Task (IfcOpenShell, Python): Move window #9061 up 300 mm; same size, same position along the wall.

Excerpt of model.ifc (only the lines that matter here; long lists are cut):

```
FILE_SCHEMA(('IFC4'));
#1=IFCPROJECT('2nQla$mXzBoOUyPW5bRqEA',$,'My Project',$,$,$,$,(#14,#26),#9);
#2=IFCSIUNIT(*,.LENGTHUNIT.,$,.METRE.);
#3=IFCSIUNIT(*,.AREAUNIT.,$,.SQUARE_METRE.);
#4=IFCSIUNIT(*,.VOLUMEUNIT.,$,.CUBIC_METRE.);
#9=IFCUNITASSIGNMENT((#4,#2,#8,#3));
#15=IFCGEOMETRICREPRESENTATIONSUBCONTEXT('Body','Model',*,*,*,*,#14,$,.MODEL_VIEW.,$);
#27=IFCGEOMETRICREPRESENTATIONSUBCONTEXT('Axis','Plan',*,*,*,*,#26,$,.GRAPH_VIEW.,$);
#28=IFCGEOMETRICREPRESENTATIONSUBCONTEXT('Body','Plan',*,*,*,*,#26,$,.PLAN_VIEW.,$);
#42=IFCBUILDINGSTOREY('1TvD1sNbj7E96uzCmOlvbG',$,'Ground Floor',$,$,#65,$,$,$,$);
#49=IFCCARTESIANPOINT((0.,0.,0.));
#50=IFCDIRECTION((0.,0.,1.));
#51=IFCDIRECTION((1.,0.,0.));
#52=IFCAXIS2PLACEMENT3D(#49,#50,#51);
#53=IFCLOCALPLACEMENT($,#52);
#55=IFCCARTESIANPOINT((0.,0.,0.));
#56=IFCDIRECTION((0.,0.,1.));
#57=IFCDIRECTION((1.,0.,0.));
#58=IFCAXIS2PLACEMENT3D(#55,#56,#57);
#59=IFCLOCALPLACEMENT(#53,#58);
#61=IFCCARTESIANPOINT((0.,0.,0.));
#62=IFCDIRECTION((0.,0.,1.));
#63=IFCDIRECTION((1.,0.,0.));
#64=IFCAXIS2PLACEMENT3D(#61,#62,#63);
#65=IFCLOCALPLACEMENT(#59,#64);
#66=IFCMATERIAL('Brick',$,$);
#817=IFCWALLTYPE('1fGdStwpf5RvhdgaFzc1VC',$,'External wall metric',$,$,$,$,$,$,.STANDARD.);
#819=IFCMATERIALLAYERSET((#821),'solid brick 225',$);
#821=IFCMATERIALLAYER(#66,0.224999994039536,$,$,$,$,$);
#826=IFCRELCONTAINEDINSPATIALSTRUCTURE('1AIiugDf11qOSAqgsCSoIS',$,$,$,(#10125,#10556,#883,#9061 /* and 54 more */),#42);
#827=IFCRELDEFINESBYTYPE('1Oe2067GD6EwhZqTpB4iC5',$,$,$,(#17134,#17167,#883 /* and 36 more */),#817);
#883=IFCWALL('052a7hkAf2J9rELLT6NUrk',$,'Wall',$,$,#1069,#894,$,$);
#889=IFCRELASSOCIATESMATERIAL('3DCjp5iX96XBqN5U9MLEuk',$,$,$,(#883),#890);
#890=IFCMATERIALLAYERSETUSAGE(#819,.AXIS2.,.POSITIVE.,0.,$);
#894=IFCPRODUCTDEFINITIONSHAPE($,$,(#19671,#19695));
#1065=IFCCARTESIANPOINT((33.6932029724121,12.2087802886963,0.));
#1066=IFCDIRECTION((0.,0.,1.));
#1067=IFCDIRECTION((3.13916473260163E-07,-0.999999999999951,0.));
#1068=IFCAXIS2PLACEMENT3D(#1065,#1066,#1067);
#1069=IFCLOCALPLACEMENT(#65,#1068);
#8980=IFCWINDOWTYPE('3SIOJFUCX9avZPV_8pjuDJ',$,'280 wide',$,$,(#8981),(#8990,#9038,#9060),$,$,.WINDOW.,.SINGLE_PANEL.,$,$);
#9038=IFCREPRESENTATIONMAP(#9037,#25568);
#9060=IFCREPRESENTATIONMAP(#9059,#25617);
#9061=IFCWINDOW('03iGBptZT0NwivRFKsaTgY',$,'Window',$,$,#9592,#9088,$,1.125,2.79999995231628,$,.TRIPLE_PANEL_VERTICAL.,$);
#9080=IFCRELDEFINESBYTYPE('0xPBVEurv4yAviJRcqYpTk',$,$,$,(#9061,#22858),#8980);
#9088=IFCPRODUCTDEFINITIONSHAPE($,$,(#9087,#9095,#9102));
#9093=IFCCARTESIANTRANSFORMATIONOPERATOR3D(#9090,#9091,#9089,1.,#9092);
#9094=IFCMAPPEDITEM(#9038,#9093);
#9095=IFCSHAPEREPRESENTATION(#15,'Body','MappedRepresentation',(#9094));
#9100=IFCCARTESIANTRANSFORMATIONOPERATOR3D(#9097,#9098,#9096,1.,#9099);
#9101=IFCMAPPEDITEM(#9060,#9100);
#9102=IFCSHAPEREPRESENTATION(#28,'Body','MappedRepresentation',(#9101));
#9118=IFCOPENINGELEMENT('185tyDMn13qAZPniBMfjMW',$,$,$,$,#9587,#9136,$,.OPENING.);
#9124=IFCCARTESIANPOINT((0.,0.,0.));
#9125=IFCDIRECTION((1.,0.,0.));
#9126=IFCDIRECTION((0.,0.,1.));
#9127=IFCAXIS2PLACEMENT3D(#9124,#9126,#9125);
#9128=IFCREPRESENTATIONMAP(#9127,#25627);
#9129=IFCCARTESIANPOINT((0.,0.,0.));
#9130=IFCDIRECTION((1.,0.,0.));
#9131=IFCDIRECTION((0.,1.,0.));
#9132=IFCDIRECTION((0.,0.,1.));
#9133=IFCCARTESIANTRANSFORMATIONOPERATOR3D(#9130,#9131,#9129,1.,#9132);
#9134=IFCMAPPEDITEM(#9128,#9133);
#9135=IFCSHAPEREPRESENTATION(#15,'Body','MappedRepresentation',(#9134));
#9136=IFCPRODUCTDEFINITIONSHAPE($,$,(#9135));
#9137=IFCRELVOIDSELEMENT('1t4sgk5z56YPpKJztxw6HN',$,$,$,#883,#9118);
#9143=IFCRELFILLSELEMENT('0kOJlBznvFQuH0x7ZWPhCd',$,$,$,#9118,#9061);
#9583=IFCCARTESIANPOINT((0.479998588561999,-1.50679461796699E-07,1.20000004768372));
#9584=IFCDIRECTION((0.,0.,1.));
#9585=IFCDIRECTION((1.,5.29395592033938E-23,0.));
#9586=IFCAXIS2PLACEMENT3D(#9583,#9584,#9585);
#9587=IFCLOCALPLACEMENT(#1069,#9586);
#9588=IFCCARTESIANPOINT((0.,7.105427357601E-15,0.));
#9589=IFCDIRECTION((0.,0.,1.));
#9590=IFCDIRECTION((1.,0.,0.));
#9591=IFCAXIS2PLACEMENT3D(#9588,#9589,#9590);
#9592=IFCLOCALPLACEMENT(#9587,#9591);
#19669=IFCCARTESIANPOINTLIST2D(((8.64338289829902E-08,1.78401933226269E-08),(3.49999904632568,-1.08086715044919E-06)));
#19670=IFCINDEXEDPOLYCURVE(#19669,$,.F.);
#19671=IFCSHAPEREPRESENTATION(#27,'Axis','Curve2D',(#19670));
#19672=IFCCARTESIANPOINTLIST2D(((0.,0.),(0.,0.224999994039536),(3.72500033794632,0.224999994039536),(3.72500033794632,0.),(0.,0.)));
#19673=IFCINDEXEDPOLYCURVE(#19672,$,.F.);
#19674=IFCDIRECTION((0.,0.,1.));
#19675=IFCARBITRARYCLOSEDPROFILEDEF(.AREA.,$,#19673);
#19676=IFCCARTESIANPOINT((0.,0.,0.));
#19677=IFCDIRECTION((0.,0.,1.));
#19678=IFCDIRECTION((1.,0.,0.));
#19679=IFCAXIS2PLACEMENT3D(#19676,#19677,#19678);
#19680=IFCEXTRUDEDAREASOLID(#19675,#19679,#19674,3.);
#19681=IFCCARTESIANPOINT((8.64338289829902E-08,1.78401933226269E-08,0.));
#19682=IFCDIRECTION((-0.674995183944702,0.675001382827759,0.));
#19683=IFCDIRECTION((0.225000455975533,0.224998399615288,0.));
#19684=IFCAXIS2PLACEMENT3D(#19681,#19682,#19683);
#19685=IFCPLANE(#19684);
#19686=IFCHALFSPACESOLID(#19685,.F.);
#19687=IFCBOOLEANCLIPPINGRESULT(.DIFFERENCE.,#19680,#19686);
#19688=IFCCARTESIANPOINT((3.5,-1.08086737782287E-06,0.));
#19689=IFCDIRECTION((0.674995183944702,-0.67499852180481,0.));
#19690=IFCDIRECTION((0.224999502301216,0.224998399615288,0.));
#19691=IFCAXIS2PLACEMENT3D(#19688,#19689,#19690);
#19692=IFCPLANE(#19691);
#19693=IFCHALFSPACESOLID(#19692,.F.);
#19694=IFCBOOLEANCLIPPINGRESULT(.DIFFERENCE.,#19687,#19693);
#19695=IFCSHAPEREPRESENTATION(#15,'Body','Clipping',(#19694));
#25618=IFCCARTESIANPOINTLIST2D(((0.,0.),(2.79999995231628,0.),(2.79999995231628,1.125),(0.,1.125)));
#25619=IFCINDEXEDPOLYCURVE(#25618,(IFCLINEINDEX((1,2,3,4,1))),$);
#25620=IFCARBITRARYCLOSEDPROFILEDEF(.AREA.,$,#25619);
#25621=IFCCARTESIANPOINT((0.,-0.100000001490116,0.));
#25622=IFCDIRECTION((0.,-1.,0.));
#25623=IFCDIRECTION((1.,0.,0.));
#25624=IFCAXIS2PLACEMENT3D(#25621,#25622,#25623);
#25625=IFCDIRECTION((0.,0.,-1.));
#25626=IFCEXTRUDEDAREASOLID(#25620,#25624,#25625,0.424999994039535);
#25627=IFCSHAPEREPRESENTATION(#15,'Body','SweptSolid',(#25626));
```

```python
import numpy as np
import ifcopenshell
import ifcopenshell.api.geometry
import ifcopenshell.util.placement
import ifcopenshell.util.unit

model = ifcopenshell.open("model.ifc")
unit_scale = ifcopenshell.util.unit.calculate_unit_scale(model)

window = model.by_id(9061)
opening = window.FillsVoids[0].RelatingOpeningElement
dz = 0.3

shift = np.array([0.0, 0.0, dz])
# The window is placed relative to its opening, so it follows when the opening moves.
matrix = ifcopenshell.util.placement.get_local_placement(opening.ObjectPlacement)
matrix[:3, 3] += shift
ifcopenshell.api.geometry.edit_object_placement(
    model, product=opening, matrix=matrix, is_si=False, should_transform_children=True
)

print(f"moved by {dz * unit_scale:+.3f} m")

model.write("model_rev.ifc")
```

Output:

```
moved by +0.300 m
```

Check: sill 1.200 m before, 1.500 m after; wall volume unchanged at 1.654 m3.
